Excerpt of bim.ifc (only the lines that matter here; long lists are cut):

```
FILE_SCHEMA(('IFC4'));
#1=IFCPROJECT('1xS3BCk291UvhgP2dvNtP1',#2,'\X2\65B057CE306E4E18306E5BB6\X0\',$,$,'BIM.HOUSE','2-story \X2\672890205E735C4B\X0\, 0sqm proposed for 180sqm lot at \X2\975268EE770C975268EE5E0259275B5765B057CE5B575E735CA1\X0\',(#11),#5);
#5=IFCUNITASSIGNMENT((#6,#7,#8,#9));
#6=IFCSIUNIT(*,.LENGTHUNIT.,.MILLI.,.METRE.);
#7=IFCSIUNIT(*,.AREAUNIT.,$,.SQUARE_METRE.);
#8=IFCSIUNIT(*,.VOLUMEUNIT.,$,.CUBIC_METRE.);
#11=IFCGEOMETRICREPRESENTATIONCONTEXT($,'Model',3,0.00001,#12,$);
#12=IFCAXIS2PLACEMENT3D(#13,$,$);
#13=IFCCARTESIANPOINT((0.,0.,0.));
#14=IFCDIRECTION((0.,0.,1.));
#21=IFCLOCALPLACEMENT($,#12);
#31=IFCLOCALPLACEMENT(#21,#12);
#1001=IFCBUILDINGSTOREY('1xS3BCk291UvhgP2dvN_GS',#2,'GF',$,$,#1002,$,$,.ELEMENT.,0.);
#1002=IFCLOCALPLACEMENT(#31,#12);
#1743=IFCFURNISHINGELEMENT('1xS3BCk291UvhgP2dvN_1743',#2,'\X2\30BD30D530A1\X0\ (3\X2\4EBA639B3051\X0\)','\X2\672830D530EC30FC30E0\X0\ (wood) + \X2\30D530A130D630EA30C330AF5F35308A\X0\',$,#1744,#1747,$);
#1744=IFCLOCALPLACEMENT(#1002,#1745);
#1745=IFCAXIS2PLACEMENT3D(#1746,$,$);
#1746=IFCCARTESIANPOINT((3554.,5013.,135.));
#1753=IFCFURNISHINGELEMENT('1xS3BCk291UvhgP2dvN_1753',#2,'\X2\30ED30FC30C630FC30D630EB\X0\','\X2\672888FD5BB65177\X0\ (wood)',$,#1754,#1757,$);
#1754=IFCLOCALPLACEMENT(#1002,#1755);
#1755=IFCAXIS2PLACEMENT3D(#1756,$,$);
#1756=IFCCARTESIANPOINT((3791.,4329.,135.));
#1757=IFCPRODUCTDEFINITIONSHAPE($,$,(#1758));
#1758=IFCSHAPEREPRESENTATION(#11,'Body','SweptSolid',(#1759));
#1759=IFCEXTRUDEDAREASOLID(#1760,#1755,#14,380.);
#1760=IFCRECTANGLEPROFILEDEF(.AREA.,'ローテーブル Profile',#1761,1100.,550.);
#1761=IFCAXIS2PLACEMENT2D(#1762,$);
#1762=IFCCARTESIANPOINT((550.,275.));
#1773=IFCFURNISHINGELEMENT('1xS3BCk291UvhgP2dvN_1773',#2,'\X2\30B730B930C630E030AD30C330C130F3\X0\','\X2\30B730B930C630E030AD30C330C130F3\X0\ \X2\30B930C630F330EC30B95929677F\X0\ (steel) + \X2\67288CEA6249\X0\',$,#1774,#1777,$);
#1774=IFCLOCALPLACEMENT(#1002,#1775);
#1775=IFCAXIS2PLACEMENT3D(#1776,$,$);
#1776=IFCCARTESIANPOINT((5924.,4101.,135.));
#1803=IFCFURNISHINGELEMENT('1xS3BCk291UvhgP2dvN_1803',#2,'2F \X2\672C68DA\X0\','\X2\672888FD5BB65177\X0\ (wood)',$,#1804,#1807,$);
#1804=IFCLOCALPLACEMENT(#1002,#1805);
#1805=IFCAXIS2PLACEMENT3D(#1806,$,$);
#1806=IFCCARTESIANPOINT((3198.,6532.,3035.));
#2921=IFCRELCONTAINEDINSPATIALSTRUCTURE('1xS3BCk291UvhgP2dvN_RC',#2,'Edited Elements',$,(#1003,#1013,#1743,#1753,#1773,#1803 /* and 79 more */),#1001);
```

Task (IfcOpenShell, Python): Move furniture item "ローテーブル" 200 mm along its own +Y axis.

```python
import ifcopenshell
import ifcopenshell.api.geometry
import ifcopenshell.util.placement

model = ifcopenshell.open("bim.ifc")

item = model.by_guid("1xS3BCk291UvhgP2dvN_1753")
matrix = ifcopenshell.util.placement.get_local_placement(item.ObjectPlacement)
matrix[:3, 3] += matrix[:3, 1] * 200.0
ifcopenshell.api.geometry.edit_object_placement(model, product=item, matrix=matrix, is_si=False)

print(ifcopenshell.util.placement.get_local_placement(item.ObjectPlacement).round(3) + 0.0)

model.write("bim-out.ifc")
```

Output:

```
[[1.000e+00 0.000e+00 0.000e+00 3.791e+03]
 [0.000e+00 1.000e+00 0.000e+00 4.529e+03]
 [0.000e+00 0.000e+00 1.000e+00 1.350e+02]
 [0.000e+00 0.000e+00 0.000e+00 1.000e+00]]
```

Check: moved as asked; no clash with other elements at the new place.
